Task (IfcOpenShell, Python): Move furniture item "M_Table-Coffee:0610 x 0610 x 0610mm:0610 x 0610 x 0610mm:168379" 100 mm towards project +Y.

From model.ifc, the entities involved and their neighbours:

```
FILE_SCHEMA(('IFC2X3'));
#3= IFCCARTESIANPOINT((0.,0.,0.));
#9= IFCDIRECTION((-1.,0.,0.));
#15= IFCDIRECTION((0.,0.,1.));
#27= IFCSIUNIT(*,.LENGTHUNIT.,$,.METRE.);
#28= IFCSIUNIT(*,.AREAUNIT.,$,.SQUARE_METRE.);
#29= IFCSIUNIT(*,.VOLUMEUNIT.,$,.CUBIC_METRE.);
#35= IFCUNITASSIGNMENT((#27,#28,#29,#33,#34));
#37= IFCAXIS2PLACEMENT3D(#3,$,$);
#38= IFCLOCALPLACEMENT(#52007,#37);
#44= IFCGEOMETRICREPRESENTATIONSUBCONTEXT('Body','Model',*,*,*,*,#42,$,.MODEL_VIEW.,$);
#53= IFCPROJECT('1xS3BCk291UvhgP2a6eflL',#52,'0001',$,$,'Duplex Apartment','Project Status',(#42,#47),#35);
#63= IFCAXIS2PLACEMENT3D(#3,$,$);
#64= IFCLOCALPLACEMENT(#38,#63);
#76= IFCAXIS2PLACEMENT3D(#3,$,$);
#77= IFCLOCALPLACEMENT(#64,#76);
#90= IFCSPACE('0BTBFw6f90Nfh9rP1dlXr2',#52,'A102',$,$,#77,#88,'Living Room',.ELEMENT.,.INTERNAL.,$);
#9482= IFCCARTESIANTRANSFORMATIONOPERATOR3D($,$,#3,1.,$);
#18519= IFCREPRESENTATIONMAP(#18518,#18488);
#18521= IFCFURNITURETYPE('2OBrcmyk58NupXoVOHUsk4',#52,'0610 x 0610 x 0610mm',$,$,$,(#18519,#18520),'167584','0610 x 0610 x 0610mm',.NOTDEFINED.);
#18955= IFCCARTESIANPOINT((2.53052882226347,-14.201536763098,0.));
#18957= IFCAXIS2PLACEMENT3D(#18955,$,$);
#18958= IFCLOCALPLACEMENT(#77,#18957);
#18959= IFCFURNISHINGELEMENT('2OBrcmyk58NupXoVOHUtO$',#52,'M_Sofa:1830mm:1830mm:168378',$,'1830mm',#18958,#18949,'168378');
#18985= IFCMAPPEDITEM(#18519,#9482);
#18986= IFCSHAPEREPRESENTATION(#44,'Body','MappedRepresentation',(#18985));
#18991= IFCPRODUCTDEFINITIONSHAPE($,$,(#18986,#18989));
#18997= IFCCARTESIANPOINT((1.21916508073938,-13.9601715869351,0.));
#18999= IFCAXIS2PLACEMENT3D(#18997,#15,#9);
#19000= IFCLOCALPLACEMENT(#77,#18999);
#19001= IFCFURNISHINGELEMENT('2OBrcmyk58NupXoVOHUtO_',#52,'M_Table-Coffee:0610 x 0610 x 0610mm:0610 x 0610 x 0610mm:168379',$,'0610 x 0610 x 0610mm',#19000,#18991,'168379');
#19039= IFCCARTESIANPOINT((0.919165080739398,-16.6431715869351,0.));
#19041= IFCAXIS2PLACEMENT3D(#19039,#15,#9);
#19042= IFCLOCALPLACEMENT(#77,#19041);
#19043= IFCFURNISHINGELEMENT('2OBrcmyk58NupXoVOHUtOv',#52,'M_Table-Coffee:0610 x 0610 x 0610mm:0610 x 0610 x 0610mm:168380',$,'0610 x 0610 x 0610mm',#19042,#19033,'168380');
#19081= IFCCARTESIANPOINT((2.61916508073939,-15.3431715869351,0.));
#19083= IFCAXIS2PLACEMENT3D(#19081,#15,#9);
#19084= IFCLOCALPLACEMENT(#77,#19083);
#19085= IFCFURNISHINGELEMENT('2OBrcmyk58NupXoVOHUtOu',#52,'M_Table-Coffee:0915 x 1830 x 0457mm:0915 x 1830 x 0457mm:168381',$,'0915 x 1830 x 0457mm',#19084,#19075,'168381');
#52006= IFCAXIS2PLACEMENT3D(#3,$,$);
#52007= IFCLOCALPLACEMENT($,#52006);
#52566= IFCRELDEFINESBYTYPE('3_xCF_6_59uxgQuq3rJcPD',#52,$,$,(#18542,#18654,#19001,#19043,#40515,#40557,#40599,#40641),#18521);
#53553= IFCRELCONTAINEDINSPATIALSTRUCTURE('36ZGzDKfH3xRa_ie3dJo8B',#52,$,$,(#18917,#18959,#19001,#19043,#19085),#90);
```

```python
import ifcopenshell
import ifcopenshell.api.geometry
import ifcopenshell.util.placement

model = ifcopenshell.open("model.ifc")

item = model.by_guid("2OBrcmyk58NupXoVOHUtO_")
matrix = ifcopenshell.util.placement.get_local_placement(item.ObjectPlacement)
matrix[1, 3] += 0.1
ifcopenshell.api.geometry.edit_object_placement(model, product=item, matrix=matrix, is_si=False)

print(ifcopenshell.util.placement.get_local_placement(item.ObjectPlacement).round(3) + 0.0)

model.write("model_updated.ifc")
```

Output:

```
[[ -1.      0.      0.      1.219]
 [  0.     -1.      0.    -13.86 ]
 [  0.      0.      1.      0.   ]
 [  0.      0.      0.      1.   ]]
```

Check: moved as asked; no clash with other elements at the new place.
